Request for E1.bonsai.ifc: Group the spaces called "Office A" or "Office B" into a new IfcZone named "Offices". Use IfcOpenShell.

First a look at what the model holds.

```python
import ifcopenshell

model = ifcopenshell.open("E1.bonsai.ifc")
print(model.schema)
seen = {}
for space in model.by_type("IfcSpace"):
    seen[space.LongName] = seen.get(space.LongName, 0) + 1
for name, count in sorted(seen.items(), key=str):
    print(count, "x", name)
print("zones:", [z.Name for z in model.by_type("IfcZone")][:20])
```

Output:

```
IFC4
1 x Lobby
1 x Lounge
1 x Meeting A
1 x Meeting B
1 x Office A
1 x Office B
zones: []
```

```python
import ifcopenshell
import ifcopenshell.api.group
import ifcopenshell.api.root

model = ifcopenshell.open("E1.bonsai.ifc")

names = {"Office A", "Office B"}
spaces = [s for s in model.by_type("IfcSpace") if s.LongName in names]

zone = ifcopenshell.api.root.create_entity(model, ifc_class="IfcZone", name="Offices")
ifcopenshell.api.group.assign_group(model, products=spaces, group=zone)
print(len(spaces), "spaces in", zone.Name)

model.write("E1.bonsai_v2.ifc")
```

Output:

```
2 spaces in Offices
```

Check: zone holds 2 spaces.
